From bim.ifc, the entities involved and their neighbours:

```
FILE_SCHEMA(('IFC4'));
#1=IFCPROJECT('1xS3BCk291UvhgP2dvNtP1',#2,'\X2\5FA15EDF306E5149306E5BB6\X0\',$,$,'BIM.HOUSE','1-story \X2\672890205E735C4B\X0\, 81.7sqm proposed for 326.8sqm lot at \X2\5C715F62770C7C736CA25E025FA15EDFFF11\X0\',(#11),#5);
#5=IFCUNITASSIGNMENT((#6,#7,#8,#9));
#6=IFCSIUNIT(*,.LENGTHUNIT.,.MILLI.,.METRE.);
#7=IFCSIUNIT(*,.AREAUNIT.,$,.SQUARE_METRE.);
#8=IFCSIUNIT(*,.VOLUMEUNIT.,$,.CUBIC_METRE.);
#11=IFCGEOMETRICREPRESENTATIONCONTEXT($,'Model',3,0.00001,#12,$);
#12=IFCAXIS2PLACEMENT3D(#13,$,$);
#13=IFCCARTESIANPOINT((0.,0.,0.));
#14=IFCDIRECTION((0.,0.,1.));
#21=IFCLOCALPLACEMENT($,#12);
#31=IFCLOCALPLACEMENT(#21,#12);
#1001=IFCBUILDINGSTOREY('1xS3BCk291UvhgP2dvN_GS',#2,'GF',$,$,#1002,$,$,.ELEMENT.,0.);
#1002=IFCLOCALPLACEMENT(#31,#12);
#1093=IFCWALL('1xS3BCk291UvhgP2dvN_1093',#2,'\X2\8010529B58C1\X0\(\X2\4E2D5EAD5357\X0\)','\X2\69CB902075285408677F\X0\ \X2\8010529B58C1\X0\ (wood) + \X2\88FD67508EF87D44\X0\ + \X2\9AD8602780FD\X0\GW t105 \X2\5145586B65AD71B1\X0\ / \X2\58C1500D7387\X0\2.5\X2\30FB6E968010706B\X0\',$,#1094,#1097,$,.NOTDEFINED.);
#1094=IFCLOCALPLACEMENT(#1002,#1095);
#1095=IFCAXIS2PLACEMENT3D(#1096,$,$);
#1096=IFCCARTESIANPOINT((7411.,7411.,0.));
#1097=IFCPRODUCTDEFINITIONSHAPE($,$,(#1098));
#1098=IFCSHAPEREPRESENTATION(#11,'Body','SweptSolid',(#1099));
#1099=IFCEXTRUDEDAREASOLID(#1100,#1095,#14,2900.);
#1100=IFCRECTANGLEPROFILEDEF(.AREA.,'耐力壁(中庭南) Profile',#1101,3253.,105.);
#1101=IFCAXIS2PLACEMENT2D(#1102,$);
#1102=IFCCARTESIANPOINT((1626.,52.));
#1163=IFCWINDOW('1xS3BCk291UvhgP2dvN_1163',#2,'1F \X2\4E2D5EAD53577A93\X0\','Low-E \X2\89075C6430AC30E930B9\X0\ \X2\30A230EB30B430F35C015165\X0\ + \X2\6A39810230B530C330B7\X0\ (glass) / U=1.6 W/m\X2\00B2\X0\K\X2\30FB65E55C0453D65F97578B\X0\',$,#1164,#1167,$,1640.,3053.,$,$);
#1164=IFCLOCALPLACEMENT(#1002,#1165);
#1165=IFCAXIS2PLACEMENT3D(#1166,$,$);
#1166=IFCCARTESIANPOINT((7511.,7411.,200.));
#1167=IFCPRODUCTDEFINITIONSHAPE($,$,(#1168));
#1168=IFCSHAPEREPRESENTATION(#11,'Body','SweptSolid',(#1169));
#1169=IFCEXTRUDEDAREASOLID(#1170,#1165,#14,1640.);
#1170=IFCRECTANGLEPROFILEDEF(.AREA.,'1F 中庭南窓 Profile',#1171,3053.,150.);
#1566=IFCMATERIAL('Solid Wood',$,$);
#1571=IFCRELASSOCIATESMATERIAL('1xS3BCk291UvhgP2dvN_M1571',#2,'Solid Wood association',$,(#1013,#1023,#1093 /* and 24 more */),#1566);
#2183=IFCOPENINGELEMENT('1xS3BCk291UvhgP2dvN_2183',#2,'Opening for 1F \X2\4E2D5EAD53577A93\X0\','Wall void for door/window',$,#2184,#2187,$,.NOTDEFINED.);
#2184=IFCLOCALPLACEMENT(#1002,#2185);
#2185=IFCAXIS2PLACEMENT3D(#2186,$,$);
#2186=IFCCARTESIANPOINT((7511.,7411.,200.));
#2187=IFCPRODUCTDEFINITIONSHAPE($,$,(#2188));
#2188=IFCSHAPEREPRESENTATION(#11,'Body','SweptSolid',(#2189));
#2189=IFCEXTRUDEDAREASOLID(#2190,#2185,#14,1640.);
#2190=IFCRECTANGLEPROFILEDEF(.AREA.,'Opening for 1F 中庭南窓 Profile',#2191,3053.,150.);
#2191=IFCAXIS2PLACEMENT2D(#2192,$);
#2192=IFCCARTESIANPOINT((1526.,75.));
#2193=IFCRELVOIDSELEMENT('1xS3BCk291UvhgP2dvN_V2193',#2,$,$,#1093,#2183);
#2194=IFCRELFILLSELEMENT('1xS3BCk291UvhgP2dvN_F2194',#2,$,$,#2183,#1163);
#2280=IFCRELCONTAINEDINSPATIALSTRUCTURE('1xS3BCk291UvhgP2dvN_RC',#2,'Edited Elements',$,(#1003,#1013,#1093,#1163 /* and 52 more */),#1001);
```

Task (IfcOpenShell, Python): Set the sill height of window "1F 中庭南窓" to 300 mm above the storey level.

```python
import numpy as np
import ifcopenshell
import ifcopenshell.api.geometry
import ifcopenshell.geom
import ifcopenshell.util.element
import ifcopenshell.util.placement
import ifcopenshell.util.shape
import ifcopenshell.util.unit

model = ifcopenshell.open("bim.ifc")
unit_scale = ifcopenshell.util.unit.calculate_unit_scale(model)

window = model.by_guid("1xS3BCk291UvhgP2dvN_1163")
opening = window.FillsVoids[0].RelatingOpeningElement
storey = ifcopenshell.util.element.get_container(window, ifc_class="IfcBuildingStorey")
level = ifcopenshell.util.placement.get_local_placement(storey.ObjectPlacement)[2, 3]

# The opening's origin need not be at the sill, so measure its lowest point.
shape = ifcopenshell.geom.create_shape(ifcopenshell.geom.settings(), opening)
bottom = ifcopenshell.util.shape.get_shape_bottom_elevation(shape, shape.geometry) / unit_scale
dz = level + 0.3 / unit_scale - bottom

shift = np.array([0.0, 0.0, dz])
# The window is not placed relative to its opening, so move both.
for product in (opening, window):
    matrix = ifcopenshell.util.placement.get_local_placement(product.ObjectPlacement)
    matrix[:3, 3] += shift
    ifcopenshell.api.geometry.edit_object_placement(model, product=product, matrix=matrix, is_si=False)

print(f"moved by {dz * unit_scale:+.3f} m")

model.write("bim_updated.ifc")
```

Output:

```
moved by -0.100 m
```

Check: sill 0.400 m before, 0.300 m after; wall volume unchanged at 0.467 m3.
